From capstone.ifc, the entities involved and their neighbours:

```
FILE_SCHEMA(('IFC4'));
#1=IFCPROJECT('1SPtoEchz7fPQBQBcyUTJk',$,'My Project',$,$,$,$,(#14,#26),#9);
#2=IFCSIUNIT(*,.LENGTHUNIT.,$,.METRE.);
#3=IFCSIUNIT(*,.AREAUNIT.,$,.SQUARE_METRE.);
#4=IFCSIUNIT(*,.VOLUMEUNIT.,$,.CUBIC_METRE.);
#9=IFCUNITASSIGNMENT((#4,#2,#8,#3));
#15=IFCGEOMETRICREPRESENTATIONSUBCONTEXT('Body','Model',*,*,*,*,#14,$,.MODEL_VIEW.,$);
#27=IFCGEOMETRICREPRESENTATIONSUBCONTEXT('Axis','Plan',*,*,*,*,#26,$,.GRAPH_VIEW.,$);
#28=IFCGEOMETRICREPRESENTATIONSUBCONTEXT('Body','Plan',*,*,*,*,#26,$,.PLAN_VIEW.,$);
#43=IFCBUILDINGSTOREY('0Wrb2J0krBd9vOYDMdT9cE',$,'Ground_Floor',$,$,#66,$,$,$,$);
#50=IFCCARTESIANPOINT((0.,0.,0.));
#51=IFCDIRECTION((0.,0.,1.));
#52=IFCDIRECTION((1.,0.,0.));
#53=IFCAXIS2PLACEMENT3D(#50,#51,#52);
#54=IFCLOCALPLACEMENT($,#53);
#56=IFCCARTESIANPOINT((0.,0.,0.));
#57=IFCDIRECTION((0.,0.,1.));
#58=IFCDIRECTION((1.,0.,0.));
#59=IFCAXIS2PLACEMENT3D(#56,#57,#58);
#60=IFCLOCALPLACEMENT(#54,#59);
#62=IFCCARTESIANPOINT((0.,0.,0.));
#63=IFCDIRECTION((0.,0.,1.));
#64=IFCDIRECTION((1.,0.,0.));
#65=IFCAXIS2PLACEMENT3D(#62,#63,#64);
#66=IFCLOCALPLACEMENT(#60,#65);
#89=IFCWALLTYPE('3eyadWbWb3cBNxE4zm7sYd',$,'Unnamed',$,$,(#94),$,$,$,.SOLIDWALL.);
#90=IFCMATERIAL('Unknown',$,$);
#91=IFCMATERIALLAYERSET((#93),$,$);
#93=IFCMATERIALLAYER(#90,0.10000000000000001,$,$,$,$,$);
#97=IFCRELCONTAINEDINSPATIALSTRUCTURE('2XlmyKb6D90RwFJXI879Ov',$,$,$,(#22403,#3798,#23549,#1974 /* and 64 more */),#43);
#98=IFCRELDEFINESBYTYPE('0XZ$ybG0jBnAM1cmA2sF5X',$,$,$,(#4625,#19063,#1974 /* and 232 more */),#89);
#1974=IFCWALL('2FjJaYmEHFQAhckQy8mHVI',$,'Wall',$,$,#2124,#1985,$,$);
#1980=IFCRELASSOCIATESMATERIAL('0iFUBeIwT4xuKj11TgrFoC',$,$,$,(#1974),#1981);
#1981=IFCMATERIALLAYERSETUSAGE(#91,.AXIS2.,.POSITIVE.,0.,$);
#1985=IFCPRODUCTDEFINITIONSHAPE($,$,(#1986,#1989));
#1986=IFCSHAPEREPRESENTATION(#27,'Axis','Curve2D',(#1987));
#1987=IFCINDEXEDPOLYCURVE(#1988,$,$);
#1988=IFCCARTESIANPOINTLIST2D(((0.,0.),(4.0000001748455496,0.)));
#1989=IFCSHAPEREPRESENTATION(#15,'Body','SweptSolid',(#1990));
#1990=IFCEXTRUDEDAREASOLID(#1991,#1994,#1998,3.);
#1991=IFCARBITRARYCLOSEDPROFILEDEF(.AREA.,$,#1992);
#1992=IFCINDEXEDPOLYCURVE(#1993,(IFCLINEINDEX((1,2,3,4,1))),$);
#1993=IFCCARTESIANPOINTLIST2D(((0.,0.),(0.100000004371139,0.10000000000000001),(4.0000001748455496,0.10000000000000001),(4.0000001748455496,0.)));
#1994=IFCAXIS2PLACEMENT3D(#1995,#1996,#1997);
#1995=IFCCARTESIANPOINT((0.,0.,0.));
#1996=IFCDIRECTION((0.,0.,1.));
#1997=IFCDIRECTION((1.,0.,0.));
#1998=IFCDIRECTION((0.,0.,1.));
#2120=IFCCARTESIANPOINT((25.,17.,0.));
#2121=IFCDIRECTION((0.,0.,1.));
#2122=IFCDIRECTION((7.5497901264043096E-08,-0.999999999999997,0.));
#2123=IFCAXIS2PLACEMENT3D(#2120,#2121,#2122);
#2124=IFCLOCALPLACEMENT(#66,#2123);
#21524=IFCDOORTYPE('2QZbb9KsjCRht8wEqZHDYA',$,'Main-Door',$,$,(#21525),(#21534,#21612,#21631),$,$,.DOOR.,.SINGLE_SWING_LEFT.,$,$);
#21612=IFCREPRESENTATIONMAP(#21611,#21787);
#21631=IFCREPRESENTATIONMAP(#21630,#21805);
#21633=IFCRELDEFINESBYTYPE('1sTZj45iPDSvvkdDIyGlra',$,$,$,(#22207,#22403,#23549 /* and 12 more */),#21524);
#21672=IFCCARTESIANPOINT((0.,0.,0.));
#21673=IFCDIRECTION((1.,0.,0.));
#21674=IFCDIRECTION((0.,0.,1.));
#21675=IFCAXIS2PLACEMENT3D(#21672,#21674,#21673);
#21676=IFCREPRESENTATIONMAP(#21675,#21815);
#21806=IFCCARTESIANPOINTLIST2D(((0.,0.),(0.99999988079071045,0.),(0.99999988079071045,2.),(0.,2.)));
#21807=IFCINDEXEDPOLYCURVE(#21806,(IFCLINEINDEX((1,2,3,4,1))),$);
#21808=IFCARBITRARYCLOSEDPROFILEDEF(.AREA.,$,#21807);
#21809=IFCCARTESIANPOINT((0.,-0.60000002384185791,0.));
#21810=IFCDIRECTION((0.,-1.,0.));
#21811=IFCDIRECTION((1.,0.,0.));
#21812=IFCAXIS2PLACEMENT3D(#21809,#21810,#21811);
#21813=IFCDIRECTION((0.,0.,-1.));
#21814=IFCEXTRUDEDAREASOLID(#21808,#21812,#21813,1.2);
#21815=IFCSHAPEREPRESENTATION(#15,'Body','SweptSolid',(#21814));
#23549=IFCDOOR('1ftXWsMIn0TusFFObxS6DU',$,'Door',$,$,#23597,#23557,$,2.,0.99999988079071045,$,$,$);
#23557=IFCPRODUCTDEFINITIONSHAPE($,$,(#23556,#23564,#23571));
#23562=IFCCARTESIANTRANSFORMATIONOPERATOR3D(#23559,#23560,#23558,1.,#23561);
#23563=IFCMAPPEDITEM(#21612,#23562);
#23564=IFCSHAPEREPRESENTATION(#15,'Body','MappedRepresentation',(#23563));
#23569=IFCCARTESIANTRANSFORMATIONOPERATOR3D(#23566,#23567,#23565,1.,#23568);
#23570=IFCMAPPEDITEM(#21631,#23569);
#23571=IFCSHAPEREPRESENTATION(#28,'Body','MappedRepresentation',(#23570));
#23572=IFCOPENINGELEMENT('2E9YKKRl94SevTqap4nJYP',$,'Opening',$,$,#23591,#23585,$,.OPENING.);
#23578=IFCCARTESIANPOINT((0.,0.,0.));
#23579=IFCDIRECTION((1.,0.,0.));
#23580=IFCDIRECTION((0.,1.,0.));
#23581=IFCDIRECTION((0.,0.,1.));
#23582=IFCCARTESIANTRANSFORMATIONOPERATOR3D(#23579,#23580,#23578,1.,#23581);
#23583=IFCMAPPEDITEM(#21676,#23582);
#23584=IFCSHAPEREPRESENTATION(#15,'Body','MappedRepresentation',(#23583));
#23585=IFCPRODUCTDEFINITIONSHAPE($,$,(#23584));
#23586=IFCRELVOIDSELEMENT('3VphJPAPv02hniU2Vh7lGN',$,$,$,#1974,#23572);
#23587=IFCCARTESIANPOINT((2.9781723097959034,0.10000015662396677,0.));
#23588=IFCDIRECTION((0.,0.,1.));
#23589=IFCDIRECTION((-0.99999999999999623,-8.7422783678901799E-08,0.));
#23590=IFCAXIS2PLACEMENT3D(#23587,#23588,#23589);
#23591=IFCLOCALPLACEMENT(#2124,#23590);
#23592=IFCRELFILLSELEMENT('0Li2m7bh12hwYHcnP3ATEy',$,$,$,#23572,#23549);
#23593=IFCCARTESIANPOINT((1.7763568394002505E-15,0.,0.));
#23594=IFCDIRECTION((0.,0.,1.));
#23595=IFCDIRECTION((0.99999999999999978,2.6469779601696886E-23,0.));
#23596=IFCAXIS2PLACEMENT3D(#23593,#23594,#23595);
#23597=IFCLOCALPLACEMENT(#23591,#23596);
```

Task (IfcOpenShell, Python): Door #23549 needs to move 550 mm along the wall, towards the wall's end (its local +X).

```python
import ifcopenshell
import ifcopenshell.api.geometry
import ifcopenshell.util.placement
import ifcopenshell.util.unit

model = ifcopenshell.open("capstone.ifc")
unit_scale = ifcopenshell.util.unit.calculate_unit_scale(model)

door = model.by_guid("1ftXWsMIn0TusFFObxS6DU")
opening = door.FillsVoids[0].RelatingOpeningElement
wall = opening.VoidsElements[0].RelatingBuildingElement

wall_matrix = ifcopenshell.util.placement.get_local_placement(wall.ObjectPlacement)
shift = wall_matrix[:3, 0] * 0.55 / unit_scale
before = ifcopenshell.util.placement.get_local_placement(door.ObjectPlacement)[:3, 3].copy()

# The door is placed relative to its opening, so it follows when the opening moves.
matrix = ifcopenshell.util.placement.get_local_placement(opening.ObjectPlacement)
matrix[:3, 3] += shift
ifcopenshell.api.geometry.edit_object_placement(
    model, product=opening, matrix=matrix, is_si=False, should_transform_children=True
)

after = ifcopenshell.util.placement.get_local_placement(door.ObjectPlacement)[:3, 3]
print("door moved by", (after - before).round(3) + 0.0)

model.write("capstone_v2.ifc")
```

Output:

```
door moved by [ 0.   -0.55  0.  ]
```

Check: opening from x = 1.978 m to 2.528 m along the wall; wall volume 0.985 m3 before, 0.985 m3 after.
